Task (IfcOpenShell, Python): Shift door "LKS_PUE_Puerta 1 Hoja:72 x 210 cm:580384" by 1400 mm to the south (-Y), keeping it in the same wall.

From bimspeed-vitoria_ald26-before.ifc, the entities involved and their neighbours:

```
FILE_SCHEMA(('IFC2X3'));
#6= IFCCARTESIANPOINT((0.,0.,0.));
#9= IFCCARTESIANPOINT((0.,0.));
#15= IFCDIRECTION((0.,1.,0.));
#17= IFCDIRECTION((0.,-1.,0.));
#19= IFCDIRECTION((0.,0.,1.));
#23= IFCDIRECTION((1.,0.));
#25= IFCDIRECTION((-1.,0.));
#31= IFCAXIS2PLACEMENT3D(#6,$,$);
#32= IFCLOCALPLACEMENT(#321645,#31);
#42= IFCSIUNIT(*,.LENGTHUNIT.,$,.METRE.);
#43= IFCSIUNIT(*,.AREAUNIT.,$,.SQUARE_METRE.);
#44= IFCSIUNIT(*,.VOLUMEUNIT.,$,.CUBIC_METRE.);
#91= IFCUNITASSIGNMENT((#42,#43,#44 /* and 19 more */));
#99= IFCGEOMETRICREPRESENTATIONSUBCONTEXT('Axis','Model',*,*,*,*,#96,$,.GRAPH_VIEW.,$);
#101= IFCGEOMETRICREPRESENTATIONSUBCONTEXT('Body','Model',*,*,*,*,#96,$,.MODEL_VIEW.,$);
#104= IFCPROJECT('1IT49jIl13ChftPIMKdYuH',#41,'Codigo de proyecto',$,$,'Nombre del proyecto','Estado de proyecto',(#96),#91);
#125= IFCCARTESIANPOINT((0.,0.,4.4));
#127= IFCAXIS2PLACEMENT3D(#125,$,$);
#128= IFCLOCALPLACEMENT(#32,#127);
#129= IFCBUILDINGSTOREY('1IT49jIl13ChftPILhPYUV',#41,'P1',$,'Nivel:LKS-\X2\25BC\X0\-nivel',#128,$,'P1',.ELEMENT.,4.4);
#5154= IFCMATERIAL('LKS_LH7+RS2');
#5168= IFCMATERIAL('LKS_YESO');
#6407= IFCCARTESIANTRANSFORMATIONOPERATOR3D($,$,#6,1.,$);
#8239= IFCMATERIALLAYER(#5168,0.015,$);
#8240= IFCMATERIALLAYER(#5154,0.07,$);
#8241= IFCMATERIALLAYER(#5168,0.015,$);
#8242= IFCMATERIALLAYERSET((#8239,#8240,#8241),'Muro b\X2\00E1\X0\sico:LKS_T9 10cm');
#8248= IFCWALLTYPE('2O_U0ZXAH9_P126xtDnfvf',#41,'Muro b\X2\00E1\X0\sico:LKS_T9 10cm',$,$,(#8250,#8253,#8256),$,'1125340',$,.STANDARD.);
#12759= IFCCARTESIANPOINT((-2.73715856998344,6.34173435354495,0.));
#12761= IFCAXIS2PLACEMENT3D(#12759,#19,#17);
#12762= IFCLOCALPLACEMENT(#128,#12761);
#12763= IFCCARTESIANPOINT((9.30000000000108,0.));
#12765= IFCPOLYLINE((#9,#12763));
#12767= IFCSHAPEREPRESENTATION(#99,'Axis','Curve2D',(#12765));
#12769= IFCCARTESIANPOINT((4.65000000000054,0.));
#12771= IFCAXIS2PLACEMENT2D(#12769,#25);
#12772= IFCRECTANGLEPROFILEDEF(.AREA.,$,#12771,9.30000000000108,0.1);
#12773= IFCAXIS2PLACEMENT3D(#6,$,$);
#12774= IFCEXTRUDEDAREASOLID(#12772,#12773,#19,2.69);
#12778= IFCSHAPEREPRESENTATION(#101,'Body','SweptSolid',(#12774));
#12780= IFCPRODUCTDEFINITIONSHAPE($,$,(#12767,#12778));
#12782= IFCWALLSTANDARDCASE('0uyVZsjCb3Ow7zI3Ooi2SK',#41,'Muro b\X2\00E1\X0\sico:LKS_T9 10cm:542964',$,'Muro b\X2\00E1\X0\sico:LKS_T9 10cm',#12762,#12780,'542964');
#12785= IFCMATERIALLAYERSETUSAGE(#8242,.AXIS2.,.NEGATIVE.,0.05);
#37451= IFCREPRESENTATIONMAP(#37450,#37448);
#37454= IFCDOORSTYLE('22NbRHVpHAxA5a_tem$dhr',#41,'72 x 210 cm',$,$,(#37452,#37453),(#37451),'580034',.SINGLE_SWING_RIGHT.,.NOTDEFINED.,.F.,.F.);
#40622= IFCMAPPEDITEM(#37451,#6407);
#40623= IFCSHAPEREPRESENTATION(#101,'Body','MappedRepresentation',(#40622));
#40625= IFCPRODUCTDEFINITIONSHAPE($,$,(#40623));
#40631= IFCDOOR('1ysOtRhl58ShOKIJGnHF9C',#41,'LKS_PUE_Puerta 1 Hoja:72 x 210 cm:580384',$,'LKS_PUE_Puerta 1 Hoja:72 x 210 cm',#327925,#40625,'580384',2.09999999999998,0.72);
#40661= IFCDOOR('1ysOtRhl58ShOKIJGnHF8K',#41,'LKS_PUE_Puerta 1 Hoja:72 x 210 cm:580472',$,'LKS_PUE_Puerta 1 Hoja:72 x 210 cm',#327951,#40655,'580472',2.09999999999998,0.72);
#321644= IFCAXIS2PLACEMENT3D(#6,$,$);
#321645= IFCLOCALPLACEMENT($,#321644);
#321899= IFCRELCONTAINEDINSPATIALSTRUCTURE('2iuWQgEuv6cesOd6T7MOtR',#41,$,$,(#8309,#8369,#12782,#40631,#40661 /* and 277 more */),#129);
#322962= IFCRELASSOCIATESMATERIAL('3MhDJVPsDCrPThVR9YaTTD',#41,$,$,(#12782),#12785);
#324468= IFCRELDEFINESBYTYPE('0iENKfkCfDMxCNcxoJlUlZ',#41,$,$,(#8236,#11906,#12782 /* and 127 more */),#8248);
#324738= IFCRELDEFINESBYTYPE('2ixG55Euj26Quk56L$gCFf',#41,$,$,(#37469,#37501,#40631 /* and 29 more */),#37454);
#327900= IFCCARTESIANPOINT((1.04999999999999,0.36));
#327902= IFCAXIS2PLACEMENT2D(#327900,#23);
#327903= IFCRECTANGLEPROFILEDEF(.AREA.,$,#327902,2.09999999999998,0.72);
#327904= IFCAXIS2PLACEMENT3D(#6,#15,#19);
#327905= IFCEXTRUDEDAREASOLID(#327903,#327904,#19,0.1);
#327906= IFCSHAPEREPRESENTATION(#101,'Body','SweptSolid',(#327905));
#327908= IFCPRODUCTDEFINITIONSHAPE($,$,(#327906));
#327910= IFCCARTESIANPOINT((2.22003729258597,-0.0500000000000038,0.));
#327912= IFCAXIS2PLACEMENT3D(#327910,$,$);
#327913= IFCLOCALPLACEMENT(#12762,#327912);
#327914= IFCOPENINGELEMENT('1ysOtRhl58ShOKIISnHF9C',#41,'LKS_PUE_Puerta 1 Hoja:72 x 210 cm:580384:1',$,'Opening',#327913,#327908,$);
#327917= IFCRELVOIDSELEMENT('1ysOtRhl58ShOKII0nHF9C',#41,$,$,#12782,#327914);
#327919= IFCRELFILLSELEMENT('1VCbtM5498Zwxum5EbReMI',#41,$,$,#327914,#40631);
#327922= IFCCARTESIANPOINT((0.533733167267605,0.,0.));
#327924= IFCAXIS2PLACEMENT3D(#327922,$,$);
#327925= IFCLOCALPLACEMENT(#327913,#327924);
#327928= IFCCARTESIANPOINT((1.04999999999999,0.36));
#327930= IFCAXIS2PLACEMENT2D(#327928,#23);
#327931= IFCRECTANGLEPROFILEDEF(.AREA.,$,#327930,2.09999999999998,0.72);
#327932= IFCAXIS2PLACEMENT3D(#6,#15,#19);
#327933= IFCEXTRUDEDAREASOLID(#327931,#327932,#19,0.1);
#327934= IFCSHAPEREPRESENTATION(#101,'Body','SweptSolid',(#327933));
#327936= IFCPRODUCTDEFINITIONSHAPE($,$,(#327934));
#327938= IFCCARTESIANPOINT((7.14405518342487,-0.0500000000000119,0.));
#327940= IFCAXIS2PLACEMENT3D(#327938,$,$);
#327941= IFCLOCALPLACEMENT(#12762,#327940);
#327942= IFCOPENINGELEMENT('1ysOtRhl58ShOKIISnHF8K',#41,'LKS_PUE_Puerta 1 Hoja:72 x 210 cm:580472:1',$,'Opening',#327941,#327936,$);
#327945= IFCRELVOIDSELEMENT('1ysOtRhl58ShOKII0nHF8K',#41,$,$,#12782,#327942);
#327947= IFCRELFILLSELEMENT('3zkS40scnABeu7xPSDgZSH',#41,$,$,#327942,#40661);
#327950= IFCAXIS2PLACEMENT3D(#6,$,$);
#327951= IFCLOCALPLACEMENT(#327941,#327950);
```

```python
import ifcopenshell
import ifcopenshell.api.geometry
import ifcopenshell.util.placement
import ifcopenshell.util.unit

model = ifcopenshell.open("bimspeed-vitoria_ald26-before.ifc")
unit_scale = ifcopenshell.util.unit.calculate_unit_scale(model)

door = model.by_id(40631)
opening = door.FillsVoids[0].RelatingOpeningElement
wall = opening.VoidsElements[0].RelatingBuildingElement

wall_matrix = ifcopenshell.util.placement.get_local_placement(wall.ObjectPlacement)
shift = wall_matrix[:3, 0] * 1.4 / unit_scale
before = ifcopenshell.util.placement.get_local_placement(door.ObjectPlacement)[:3, 3].copy()

# The door is placed relative to its opening, so it follows when the opening moves.
matrix = ifcopenshell.util.placement.get_local_placement(opening.ObjectPlacement)
matrix[:3, 3] += shift
ifcopenshell.api.geometry.edit_object_placement(
    model, product=opening, matrix=matrix, is_si=False, should_transform_children=True
)

after = ifcopenshell.util.placement.get_local_placement(door.ObjectPlacement)[:3, 3]
print("door moved by", (after - before).round(3) + 0.0)

model.write("bimspeed-vitoria_ald26-before-out.ifc")
```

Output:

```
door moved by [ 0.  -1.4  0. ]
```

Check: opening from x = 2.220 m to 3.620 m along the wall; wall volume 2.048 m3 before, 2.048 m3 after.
